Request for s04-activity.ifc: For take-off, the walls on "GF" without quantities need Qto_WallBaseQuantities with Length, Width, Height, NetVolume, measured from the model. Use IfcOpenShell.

First a look at what the model holds.

```python
import ifcopenshell
import ifcopenshell.util.element
import ifcopenshell.util.unit

model = ifcopenshell.open("s04-activity.ifc")
print(model.schema)
for unit_type in ("LENGTHUNIT", "AREAUNIT", "VOLUMEUNIT"):
    print(unit_type, ifcopenshell.util.unit.calculate_unit_scale(model, unit_type))
storey = next(s for s in model.by_type("IfcBuildingStorey") if s.Name == "GF")
walls = [e for e in ifcopenshell.util.element.get_decomposition(storey) if e.is_a("IfcWall")]
for e in sorted(walls, key=lambda e: e.id()):
    print(e.id(), e.is_a(), e.Name, list(ifcopenshell.util.element.get_psets(e, qtos_only=True)), sep=" | ")
```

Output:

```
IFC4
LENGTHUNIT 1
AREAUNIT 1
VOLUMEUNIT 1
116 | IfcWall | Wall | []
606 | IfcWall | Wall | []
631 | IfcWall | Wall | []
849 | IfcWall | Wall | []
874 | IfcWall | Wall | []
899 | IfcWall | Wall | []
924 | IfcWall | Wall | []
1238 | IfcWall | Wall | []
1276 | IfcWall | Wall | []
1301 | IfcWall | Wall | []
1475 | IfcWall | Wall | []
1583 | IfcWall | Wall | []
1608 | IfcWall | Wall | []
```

```python
import ifcopenshell
import ifcopenshell.api.pset
import ifcopenshell.geom
import ifcopenshell.util.element
import ifcopenshell.util.shape
import ifcopenshell.util.unit

model = ifcopenshell.open("s04-activity.ifc")
unit_scale = ifcopenshell.util.unit.calculate_unit_scale(model)
volume_scale = ifcopenshell.util.unit.calculate_unit_scale(model, "VOLUMEUNIT")
settings = ifcopenshell.geom.settings()

storey = next(s for s in model.by_type("IfcBuildingStorey") if s.Name == "GF")
walls = [e for e in ifcopenshell.util.element.get_decomposition(storey) if e.is_a("IfcWall")]

for e in sorted(walls, key=lambda e: e.id()):
    if ifcopenshell.util.element.get_psets(e, qtos_only=True, should_inherit=False):
        continue
    # Geometry comes back in metres, in the element's own axes.
    shape = ifcopenshell.geom.create_shape(settings, e)
    values = {
        "Length": ifcopenshell.util.shape.get_x(shape.geometry) / unit_scale,
        "Width": ifcopenshell.util.shape.get_y(shape.geometry) / unit_scale,
        "Height": ifcopenshell.util.shape.get_z(shape.geometry) / unit_scale,
        "NetVolume": ifcopenshell.util.shape.get_volume(shape.geometry) / volume_scale,
    }
    qto = ifcopenshell.api.pset.add_qto(model, product=e, name="Qto_WallBaseQuantities")
    ifcopenshell.api.pset.edit_qto(model, qto=qto, properties=values)
    print(e.id(), {k: round(v, 3) for k, v in values.items()})

model.write("s04-activity_updated.ifc")
```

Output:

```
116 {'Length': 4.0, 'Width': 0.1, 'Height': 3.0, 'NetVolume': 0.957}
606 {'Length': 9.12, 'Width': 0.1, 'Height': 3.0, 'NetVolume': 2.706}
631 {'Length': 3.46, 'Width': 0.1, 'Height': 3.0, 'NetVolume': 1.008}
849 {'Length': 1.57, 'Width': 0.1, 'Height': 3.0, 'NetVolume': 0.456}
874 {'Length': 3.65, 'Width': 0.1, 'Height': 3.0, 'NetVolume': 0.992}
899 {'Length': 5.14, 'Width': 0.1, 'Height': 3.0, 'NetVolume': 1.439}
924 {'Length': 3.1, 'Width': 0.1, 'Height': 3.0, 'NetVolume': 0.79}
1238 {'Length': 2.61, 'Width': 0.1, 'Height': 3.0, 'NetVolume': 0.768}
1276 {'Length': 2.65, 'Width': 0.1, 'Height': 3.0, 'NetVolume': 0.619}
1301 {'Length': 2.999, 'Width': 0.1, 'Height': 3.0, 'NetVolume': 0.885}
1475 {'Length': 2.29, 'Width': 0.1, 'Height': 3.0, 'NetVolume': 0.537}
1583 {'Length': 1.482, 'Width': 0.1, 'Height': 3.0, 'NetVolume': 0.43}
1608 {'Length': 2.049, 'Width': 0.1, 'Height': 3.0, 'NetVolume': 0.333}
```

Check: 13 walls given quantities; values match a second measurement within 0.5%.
